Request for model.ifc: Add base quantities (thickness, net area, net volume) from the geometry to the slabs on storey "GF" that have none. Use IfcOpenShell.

First a look at what the model holds.

```python
import ifcopenshell
import ifcopenshell.util.element
import ifcopenshell.util.unit

model = ifcopenshell.open("model.ifc")
print(model.schema)
for unit_type in ("LENGTHUNIT", "AREAUNIT", "VOLUMEUNIT"):
    print(unit_type, ifcopenshell.util.unit.calculate_unit_scale(model, unit_type))
storey = next(s for s in model.by_type("IfcBuildingStorey") if s.Name == "GF")
slabs = [e for e in ifcopenshell.util.element.get_decomposition(storey) if e.is_a("IfcSlab")]
for e in sorted(slabs, key=lambda e: e.id()):
    print(e.id(), e.is_a(), e.Name, list(ifcopenshell.util.element.get_psets(e, qtos_only=True)), sep=" | ")
```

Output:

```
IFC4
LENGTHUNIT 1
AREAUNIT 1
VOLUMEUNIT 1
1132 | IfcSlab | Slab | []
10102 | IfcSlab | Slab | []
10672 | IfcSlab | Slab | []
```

```python
import ifcopenshell
import ifcopenshell.api.pset
import ifcopenshell.geom
import ifcopenshell.util.element
import ifcopenshell.util.shape
import ifcopenshell.util.unit

model = ifcopenshell.open("model.ifc")
unit_scale = ifcopenshell.util.unit.calculate_unit_scale(model)
area_scale = ifcopenshell.util.unit.calculate_unit_scale(model, "AREAUNIT")
volume_scale = ifcopenshell.util.unit.calculate_unit_scale(model, "VOLUMEUNIT")
settings = ifcopenshell.geom.settings()

storey = next(s for s in model.by_type("IfcBuildingStorey") if s.Name == "GF")
slabs = [e for e in ifcopenshell.util.element.get_decomposition(storey) if e.is_a("IfcSlab")]

for e in sorted(slabs, key=lambda e: e.id()):
    if ifcopenshell.util.element.get_psets(e, qtos_only=True, should_inherit=False):
        continue
    # Geometry comes back in metres, in the element's own axes.
    shape = ifcopenshell.geom.create_shape(settings, e)
    values = {
        "Width": ifcopenshell.util.shape.get_z(shape.geometry) / unit_scale,
        "NetArea": ifcopenshell.util.shape.get_footprint_area(shape.geometry) / area_scale,
        "NetVolume": ifcopenshell.util.shape.get_volume(shape.geometry) / volume_scale,
    }
    qto = ifcopenshell.api.pset.add_qto(model, product=e, name="Qto_SlabBaseQuantities")
    ifcopenshell.api.pset.edit_qto(model, qto=qto, properties=values)
    print(e.id(), {k: round(v, 3) for k, v in values.items()})

model.write("model-out.ifc")
```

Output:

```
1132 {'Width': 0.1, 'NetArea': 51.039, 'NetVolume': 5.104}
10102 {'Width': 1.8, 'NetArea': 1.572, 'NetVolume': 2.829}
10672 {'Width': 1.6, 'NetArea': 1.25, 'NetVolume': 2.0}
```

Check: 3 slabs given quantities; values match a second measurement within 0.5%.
